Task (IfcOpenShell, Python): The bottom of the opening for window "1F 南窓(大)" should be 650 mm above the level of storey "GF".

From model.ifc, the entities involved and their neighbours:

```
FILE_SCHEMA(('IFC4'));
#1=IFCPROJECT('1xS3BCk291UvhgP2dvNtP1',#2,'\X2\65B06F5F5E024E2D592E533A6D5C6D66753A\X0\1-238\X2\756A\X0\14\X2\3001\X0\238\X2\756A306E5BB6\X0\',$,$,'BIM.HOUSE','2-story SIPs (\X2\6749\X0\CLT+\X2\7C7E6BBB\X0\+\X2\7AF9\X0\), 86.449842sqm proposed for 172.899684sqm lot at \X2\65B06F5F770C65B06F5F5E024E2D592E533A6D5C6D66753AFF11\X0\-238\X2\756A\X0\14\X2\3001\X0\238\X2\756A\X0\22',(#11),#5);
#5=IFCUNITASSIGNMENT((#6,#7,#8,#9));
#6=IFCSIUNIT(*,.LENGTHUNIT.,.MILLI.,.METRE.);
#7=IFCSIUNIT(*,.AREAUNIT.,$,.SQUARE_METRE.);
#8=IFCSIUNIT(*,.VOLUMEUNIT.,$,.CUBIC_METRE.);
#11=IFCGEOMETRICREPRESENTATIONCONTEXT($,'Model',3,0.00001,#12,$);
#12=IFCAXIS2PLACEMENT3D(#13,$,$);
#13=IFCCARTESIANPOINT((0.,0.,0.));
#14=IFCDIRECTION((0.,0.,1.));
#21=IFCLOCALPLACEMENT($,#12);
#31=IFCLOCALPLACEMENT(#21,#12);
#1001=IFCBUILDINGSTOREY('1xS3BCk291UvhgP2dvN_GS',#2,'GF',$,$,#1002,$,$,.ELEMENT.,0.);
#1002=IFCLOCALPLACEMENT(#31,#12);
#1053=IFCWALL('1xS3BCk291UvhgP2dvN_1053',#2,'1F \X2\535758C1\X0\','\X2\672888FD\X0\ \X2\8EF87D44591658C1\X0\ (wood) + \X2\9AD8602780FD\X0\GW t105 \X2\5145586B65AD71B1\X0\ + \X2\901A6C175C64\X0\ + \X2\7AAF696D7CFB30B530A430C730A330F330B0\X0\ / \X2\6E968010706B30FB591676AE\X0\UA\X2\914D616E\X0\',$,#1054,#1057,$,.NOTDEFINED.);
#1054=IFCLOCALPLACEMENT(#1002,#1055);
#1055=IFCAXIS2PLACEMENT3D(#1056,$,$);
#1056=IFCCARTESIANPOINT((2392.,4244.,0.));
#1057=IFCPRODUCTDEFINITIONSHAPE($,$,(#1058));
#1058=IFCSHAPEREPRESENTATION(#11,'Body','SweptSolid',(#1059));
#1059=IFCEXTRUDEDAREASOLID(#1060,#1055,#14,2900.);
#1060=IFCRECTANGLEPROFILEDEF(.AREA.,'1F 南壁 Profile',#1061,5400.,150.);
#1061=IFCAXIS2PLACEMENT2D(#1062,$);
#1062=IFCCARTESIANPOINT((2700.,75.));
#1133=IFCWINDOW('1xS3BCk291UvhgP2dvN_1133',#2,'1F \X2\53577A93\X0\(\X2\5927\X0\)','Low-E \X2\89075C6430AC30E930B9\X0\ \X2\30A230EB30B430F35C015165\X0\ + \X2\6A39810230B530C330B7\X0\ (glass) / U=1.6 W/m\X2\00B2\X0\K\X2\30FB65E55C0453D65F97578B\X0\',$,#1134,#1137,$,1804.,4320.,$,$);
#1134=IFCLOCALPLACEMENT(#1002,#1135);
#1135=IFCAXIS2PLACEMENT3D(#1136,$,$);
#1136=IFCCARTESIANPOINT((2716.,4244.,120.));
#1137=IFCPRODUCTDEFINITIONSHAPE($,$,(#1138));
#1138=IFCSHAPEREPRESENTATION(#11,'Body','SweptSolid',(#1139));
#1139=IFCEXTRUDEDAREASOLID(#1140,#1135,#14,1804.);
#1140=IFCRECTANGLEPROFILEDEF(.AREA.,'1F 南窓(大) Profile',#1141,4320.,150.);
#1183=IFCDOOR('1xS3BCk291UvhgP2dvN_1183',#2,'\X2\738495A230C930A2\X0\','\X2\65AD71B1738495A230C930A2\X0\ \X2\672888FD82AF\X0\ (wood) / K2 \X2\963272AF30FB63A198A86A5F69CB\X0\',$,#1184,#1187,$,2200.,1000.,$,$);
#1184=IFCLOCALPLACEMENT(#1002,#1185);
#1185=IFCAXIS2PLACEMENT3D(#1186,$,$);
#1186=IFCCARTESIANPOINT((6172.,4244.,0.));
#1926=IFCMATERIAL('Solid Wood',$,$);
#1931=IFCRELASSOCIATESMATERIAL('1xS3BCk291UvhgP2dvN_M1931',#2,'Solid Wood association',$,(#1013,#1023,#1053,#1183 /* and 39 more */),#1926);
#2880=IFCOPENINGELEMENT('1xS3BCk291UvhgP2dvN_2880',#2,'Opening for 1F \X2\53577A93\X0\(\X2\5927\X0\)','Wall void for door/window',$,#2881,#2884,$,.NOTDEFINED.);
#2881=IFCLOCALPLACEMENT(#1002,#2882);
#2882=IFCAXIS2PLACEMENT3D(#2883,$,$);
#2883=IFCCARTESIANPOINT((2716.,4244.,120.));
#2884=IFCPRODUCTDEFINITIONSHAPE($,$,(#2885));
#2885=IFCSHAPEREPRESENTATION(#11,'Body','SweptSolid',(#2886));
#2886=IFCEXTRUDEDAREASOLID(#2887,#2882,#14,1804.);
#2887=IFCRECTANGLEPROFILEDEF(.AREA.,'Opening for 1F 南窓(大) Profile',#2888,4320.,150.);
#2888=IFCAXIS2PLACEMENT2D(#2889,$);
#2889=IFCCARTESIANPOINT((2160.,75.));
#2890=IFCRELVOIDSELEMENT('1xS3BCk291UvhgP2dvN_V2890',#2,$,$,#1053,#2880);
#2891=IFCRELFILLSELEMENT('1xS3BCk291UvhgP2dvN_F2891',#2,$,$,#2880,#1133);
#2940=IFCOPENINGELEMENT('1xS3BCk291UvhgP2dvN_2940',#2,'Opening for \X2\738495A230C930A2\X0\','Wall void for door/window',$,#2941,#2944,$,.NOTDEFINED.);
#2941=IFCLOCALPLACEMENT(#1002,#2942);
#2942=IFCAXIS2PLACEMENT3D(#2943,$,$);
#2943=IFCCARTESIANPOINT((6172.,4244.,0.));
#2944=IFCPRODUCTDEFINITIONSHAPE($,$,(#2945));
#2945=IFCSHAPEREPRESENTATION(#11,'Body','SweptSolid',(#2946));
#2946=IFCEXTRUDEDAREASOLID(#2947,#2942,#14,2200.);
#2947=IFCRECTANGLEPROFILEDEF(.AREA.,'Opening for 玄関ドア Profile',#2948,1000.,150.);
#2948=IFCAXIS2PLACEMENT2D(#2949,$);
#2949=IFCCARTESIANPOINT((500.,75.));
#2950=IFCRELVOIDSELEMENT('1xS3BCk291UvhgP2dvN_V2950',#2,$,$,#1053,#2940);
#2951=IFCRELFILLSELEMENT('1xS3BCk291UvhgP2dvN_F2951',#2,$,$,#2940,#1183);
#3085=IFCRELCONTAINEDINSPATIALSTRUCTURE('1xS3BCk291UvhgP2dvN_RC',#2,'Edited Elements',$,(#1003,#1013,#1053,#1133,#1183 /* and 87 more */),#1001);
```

```python
import numpy as np
import ifcopenshell
import ifcopenshell.api.geometry
import ifcopenshell.geom
import ifcopenshell.util.element
import ifcopenshell.util.placement
import ifcopenshell.util.shape
import ifcopenshell.util.unit

model = ifcopenshell.open("model.ifc")
unit_scale = ifcopenshell.util.unit.calculate_unit_scale(model)

window = model.by_id(1133)
opening = window.FillsVoids[0].RelatingOpeningElement
storey = ifcopenshell.util.element.get_container(window, ifc_class="IfcBuildingStorey")
level = ifcopenshell.util.placement.get_local_placement(storey.ObjectPlacement)[2, 3]

# The opening's origin need not be at the sill, so measure its lowest point.
shape = ifcopenshell.geom.create_shape(ifcopenshell.geom.settings(), opening)
bottom = ifcopenshell.util.shape.get_shape_bottom_elevation(shape, shape.geometry) / unit_scale
dz = level + 650.0 - bottom

shift = np.array([0.0, 0.0, dz])
# The window is not placed relative to its opening, so move both.
for product in (opening, window):
    matrix = ifcopenshell.util.placement.get_local_placement(product.ObjectPlacement)
    matrix[:3, 3] += shift
    ifcopenshell.api.geometry.edit_object_placement(model, product=product, matrix=matrix, is_si=False)

print(f"moved by {dz * unit_scale:+.3f} m")

model.write("model_v2.ifc")
```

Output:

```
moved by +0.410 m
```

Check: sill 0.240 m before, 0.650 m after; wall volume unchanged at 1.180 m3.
